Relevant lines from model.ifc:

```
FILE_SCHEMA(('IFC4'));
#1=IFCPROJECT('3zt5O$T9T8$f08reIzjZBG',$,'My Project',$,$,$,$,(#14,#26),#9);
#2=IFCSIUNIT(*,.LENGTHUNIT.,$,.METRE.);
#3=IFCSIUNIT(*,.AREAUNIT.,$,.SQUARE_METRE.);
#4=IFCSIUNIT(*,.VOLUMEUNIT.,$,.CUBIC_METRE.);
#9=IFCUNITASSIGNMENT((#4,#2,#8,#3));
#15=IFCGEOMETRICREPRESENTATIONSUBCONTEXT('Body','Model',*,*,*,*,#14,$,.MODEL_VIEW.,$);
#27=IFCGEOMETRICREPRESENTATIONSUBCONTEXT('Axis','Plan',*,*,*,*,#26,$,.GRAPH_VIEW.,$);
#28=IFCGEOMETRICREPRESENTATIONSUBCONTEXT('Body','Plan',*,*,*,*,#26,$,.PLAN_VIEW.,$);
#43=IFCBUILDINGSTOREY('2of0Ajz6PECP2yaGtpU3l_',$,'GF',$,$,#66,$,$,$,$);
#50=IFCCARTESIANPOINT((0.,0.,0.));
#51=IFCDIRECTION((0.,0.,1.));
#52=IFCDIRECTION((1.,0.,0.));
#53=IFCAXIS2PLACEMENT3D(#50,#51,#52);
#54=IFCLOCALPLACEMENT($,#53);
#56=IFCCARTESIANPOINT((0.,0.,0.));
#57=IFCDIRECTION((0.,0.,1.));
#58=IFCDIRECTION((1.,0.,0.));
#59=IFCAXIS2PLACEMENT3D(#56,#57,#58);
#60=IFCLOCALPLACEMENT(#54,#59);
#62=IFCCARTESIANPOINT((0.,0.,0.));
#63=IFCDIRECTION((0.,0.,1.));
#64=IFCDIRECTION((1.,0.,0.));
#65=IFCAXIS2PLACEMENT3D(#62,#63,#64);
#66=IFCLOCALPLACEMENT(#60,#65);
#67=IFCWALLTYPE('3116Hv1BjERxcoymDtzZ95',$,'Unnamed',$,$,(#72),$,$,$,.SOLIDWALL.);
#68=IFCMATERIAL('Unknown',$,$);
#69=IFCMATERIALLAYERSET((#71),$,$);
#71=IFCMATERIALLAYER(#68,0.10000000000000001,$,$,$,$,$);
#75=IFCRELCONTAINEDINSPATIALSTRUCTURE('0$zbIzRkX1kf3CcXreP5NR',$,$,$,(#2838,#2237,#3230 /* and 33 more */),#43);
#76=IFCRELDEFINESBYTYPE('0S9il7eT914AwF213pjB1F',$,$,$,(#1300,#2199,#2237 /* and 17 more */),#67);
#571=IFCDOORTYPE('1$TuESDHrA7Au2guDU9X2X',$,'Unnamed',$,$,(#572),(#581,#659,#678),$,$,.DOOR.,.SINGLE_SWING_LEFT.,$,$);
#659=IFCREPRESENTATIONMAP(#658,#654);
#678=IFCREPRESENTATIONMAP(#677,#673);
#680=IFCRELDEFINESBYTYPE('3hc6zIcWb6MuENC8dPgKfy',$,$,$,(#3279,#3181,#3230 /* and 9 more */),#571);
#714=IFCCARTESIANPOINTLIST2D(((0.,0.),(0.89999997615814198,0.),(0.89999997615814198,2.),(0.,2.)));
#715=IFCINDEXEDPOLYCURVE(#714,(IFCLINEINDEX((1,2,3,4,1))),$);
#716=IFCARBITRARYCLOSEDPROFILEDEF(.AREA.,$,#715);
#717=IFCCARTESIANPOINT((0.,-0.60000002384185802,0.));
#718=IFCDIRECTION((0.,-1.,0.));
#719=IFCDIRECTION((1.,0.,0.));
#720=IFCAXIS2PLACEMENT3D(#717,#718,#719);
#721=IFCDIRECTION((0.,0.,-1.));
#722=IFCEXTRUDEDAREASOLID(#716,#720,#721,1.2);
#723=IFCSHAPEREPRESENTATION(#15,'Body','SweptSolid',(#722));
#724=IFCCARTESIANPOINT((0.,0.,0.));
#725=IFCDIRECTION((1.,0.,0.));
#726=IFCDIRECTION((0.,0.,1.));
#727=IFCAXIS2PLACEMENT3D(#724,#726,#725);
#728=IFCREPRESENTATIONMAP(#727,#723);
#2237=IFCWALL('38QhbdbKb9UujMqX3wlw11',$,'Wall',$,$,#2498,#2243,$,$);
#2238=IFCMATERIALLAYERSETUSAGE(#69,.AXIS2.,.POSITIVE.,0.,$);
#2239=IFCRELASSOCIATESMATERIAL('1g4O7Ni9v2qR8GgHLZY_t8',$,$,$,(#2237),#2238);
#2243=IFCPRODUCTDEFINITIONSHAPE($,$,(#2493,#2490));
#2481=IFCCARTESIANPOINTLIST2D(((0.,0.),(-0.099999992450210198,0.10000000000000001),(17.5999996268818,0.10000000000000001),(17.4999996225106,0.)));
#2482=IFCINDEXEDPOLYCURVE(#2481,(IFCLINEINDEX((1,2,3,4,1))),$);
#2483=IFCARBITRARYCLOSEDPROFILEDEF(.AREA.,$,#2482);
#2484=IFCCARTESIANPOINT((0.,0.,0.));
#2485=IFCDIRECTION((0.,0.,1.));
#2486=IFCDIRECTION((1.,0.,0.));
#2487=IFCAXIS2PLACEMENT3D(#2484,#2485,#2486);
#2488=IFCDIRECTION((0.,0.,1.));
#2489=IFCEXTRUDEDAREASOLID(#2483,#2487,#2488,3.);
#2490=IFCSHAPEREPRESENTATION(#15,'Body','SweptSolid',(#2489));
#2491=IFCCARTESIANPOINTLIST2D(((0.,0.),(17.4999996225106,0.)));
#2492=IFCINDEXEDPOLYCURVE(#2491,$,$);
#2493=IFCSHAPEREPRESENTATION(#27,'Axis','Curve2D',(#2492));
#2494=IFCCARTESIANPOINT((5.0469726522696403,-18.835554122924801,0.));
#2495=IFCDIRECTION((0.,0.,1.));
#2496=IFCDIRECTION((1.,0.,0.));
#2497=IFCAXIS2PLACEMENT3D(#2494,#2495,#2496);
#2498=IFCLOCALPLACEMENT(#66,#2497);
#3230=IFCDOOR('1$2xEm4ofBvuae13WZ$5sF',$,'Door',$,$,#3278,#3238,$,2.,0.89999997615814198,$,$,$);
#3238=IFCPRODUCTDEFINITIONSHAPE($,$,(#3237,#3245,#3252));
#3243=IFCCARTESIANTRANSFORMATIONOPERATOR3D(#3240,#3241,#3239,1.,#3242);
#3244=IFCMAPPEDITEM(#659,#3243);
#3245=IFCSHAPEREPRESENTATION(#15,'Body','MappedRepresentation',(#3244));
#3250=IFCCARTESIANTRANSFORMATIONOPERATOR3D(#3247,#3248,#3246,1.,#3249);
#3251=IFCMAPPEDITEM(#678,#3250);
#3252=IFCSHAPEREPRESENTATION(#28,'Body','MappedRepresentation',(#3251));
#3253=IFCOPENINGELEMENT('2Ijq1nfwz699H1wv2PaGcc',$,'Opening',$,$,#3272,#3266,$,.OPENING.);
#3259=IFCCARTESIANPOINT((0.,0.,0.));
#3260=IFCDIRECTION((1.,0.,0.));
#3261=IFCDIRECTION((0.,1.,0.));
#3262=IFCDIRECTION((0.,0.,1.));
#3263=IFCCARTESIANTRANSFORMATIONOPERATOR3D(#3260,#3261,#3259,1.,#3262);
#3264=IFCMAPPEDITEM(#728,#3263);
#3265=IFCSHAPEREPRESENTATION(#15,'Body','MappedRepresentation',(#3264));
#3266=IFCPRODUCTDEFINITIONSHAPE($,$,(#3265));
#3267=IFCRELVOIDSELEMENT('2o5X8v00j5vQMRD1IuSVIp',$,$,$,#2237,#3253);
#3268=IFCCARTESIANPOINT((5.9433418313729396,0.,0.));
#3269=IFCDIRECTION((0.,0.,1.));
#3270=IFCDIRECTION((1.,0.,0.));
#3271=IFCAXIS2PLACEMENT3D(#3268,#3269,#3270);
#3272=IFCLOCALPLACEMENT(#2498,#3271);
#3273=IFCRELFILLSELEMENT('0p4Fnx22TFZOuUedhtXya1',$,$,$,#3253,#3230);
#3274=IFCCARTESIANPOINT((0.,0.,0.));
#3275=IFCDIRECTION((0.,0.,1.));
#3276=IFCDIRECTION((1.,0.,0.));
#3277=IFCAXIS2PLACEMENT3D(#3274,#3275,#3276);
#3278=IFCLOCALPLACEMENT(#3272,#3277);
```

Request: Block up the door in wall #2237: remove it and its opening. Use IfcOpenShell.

```python
import ifcopenshell
import ifcopenshell.api.feature
import ifcopenshell.api.root
import ifcopenshell.geom
import ifcopenshell.util.shape

model = ifcopenshell.open("model.ifc")
settings = ifcopenshell.geom.settings()


def volume(element):
    """Net volume in cubic metres, openings subtracted."""
    shape = ifcopenshell.geom.create_shape(settings, element)
    return ifcopenshell.util.shape.get_volume(shape.geometry)


door = model.by_id(3230)
opening = door.FillsVoids[0].RelatingOpeningElement
wall = opening.VoidsElements[0].RelatingBuildingElement
before = volume(wall)

ifcopenshell.api.root.remove_product(model, product=door)
ifcopenshell.api.feature.remove_feature(model, feature=opening)

after = volume(wall)

print(f"wall volume {before:.3f} -> {after:.3f} m3")

model.write("model_v2.ifc")
```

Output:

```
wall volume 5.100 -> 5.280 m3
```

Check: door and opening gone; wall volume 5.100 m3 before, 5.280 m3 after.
